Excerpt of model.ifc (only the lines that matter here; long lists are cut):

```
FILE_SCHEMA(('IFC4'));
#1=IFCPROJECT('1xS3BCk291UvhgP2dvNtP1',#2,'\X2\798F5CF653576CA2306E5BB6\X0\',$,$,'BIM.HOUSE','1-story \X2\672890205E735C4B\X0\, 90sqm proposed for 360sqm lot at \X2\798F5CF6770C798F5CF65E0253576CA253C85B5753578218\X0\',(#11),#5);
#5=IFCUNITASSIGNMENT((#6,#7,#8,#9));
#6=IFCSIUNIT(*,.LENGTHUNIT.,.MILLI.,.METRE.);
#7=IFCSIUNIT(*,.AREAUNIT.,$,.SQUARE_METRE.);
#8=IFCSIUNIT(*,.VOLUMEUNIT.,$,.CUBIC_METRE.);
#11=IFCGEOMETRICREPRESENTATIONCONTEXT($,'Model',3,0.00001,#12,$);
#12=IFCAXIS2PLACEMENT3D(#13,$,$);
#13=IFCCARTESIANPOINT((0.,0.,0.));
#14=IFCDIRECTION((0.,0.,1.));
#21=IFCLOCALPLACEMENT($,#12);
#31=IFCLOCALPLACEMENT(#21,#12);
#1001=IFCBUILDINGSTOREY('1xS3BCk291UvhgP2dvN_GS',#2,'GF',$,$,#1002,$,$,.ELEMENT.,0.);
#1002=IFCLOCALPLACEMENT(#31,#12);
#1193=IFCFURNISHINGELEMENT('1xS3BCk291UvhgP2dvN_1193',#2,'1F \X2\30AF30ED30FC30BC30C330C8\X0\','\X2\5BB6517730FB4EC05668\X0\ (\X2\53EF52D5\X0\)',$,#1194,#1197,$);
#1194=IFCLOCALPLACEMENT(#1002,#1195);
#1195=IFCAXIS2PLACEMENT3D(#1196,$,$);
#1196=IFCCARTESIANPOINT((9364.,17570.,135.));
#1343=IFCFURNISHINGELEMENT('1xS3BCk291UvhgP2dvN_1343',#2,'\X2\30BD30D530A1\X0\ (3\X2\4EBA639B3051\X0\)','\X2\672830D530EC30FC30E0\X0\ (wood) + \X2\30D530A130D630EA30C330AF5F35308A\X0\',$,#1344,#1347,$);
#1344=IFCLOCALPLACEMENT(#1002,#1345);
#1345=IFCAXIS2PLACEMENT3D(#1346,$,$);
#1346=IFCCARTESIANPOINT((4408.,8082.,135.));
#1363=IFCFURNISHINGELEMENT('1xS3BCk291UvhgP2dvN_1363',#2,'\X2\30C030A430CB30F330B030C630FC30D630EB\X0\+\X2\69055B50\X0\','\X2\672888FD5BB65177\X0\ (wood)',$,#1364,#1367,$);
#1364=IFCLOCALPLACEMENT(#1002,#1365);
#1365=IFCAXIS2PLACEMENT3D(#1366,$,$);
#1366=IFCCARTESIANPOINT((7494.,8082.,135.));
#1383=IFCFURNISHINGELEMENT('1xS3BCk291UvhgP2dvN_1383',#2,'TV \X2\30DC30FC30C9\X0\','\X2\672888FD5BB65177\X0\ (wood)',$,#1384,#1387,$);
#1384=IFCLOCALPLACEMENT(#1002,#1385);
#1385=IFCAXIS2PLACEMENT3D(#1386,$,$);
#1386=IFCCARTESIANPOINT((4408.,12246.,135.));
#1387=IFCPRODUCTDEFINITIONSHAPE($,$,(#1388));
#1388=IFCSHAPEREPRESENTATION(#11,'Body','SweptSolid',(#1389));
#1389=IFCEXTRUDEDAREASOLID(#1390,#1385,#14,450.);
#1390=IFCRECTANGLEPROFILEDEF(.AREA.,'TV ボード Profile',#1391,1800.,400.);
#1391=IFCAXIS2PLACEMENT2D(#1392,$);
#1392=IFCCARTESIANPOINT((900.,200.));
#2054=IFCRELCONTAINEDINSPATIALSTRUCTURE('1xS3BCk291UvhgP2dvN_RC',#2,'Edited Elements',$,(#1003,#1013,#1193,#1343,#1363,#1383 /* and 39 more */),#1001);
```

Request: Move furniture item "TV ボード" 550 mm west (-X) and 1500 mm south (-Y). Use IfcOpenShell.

```python
import ifcopenshell
import ifcopenshell.api.geometry
import ifcopenshell.util.placement

model = ifcopenshell.open("model.ifc")

item = model.by_guid("1xS3BCk291UvhgP2dvN_1383")
matrix = ifcopenshell.util.placement.get_local_placement(item.ObjectPlacement)
matrix[0, 3] -= 550.0
matrix[1, 3] -= 1500.0
ifcopenshell.api.geometry.edit_object_placement(model, product=item, matrix=matrix, is_si=False)

print(ifcopenshell.util.placement.get_local_placement(item.ObjectPlacement).round(3) + 0.0)

model.write("model_v2.ifc")
```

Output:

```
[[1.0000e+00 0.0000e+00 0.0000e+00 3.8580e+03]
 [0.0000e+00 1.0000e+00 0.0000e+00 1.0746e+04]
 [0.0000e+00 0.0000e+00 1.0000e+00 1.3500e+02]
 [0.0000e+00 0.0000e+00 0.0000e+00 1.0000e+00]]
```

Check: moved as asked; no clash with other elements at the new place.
